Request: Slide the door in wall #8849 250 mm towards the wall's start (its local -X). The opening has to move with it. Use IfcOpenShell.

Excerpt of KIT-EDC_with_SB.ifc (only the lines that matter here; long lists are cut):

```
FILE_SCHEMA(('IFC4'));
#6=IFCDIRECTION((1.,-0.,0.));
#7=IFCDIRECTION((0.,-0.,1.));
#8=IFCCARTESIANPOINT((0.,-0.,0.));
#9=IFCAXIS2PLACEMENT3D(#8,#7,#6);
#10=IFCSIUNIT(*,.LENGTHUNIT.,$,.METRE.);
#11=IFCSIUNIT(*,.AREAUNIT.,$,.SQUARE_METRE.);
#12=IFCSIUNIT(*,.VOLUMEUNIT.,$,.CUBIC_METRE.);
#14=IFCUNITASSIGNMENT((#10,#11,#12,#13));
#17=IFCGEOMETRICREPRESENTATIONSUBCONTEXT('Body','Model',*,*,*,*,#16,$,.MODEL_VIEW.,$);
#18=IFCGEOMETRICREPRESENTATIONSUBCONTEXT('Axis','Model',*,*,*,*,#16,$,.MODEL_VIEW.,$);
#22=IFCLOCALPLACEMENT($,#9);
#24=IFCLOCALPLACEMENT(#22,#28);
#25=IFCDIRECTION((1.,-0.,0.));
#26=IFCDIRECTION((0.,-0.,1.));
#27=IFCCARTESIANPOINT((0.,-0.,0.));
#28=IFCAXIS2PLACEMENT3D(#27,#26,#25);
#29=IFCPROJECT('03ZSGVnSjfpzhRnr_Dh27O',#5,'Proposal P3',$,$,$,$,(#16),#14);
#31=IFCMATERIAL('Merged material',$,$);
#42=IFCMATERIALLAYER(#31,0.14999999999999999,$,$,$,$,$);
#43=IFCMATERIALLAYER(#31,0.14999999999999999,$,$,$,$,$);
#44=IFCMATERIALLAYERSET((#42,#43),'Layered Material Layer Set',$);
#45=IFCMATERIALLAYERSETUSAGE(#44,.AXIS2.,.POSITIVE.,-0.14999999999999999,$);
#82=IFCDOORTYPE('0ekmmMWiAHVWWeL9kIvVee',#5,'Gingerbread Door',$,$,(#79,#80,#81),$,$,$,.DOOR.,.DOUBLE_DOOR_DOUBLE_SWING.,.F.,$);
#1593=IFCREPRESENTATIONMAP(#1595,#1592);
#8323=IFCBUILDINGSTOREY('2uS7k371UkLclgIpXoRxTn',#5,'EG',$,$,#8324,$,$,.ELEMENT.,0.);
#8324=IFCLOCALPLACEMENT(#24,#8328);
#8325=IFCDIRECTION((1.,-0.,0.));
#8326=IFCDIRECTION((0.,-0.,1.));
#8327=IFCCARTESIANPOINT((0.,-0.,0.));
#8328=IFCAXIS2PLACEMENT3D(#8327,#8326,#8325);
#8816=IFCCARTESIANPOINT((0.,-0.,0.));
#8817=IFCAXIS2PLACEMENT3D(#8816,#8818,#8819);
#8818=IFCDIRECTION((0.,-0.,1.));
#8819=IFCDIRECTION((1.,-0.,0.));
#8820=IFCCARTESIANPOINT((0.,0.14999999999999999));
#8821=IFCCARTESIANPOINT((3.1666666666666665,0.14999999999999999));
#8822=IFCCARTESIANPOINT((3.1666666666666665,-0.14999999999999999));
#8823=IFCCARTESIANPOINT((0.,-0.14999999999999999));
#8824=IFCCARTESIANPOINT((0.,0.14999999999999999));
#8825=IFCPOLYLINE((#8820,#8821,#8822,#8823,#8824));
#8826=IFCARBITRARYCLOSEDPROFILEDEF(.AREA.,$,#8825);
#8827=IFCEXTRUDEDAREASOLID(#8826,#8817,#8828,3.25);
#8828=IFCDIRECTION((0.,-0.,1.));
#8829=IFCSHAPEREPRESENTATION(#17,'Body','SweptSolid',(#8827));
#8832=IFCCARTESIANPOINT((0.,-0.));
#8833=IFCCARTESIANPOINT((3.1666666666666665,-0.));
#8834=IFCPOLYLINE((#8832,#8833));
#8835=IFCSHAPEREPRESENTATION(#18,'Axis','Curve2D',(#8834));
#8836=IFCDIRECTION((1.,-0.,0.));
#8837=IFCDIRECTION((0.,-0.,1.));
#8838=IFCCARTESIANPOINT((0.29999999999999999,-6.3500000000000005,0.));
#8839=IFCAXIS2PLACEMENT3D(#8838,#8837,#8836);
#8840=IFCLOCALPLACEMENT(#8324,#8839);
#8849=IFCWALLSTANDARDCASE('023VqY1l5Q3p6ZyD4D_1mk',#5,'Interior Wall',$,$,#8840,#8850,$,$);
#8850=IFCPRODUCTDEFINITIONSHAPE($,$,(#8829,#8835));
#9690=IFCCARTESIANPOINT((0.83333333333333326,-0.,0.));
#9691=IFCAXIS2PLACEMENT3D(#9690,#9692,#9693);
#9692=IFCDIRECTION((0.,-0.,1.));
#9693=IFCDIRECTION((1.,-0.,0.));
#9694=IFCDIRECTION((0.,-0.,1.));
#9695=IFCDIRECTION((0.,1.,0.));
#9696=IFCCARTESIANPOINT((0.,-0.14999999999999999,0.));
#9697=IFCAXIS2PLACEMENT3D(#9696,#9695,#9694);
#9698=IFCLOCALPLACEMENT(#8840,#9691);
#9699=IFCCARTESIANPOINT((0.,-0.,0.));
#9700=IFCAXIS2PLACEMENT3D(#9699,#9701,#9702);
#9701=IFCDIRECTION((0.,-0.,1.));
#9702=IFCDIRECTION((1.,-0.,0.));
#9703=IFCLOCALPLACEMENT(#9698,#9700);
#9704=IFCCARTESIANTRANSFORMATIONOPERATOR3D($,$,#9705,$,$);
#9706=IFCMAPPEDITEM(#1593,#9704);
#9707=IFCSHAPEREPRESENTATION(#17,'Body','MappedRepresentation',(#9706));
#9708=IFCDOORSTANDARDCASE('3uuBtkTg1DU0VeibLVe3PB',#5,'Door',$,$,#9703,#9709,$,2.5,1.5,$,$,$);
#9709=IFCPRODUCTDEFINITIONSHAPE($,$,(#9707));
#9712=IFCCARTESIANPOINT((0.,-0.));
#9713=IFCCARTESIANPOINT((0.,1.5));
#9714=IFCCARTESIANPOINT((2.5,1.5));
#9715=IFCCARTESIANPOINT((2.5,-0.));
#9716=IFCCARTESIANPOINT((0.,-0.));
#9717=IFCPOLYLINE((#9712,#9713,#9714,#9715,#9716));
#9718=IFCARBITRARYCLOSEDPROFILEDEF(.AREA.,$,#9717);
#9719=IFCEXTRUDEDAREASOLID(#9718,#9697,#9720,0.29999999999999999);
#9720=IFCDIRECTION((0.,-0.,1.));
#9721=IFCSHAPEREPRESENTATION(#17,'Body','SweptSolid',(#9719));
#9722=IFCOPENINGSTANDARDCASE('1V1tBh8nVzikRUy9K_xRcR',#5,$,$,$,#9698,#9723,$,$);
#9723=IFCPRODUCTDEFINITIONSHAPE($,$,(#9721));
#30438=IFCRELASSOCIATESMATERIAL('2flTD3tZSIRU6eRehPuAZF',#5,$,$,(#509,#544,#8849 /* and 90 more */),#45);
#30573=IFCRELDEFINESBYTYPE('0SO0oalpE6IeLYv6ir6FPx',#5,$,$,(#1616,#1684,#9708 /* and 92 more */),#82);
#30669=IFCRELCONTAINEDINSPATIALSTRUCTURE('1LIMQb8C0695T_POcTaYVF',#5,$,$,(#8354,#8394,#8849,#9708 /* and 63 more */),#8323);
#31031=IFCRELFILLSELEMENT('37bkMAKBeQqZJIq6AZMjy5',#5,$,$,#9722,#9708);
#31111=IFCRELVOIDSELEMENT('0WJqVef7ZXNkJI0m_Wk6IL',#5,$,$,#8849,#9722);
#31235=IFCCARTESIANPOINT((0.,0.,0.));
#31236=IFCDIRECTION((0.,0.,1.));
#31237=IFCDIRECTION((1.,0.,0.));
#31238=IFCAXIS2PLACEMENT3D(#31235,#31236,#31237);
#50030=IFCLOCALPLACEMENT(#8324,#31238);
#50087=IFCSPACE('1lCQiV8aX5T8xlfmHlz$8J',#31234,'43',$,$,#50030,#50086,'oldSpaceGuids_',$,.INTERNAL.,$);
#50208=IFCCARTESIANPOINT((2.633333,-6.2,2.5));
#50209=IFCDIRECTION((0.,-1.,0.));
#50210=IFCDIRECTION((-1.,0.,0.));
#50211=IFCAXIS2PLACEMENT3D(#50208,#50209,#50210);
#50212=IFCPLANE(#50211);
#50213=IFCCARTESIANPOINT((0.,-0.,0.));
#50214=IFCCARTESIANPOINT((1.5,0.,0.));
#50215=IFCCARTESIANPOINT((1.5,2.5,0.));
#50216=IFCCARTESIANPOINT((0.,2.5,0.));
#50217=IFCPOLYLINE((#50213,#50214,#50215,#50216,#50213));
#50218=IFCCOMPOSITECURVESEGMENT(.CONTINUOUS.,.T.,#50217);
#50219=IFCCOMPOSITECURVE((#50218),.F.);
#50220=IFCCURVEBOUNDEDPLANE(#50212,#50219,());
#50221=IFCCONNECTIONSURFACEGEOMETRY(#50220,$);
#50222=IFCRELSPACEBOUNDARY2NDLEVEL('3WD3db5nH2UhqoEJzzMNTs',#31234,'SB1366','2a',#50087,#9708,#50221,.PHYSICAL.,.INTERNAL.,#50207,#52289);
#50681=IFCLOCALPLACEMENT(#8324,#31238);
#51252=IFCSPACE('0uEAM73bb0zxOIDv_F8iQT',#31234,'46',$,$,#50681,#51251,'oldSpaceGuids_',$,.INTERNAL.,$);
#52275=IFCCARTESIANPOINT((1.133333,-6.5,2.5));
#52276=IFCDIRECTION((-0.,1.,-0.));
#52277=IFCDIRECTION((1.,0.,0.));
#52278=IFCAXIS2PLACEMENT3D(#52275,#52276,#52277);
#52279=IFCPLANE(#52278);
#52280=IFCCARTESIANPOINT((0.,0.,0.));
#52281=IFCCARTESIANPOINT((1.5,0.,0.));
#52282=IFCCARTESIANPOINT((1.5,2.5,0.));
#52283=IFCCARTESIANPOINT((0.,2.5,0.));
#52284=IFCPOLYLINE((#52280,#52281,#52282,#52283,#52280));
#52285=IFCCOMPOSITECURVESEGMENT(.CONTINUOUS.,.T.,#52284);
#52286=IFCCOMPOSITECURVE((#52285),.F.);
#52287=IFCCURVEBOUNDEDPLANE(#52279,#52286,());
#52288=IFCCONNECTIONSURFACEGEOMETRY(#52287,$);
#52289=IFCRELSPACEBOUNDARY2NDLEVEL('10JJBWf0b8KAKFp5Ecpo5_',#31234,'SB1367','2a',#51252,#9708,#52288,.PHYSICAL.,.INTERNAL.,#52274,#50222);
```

```python
import numpy as np
import ifcopenshell
import ifcopenshell.api.geometry
import ifcopenshell.util.placement

model = ifcopenshell.open("KIT-EDC_with_SB.ifc")

door = model.by_id(9708)
opening = door.FillsVoids[0].RelatingOpeningElement
wall = opening.VoidsElements[0].RelatingBuildingElement

wall_matrix = ifcopenshell.util.placement.get_local_placement(wall.ObjectPlacement)
shift = wall_matrix[:3, 0] * -0.25
before = ifcopenshell.util.placement.get_local_placement(door.ObjectPlacement)[:3, 3].copy()

# The door is placed relative to its opening, so it follows when the opening moves.
matrix = ifcopenshell.util.placement.get_local_placement(opening.ObjectPlacement)
matrix[:3, 3] += shift
ifcopenshell.api.geometry.edit_object_placement(
    model, product=opening, matrix=matrix, is_si=False, should_transform_children=True
)

# Space boundary surfaces are stored in each space's coordinates; move them too.
for rel in door.ProvidesBoundaries:
    if not rel.ConnectionGeometry:
        continue
    surface = rel.ConnectionGeometry.SurfaceOnRelatingElement.BasisSurface
    space_matrix = ifcopenshell.util.placement.get_local_placement(rel.RelatingSpace.ObjectPlacement)
    point = np.array(surface.Position.Location.Coordinates) + space_matrix[:3, :3].T @ shift
    surface.Position = model.createIfcAxis2Placement3D(
        model.createIfcCartesianPoint(point.tolist()), surface.Position.Axis, surface.Position.RefDirection
    )

after = ifcopenshell.util.placement.get_local_placement(door.ObjectPlacement)[:3, 3]
print("door moved by", (after - before).round(3) + 0.0)

model.write("KIT-EDC_with_SB_rev.ifc")
```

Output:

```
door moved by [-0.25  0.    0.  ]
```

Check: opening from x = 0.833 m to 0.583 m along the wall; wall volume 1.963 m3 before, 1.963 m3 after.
